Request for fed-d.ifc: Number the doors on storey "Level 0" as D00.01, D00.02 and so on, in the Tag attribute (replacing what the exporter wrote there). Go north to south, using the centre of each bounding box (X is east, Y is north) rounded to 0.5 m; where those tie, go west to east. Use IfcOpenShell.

First a look at what the model holds.

```python
import ifcopenshell
import ifcopenshell.util.element
import ifcopenshell.util.placement

model = ifcopenshell.open("fed-d.ifc")
print(model.schema)
storey = next(s for s in model.by_type("IfcBuildingStorey") if s.Name == "Level 0")
doors = [e for e in ifcopenshell.util.element.get_decomposition(storey) if e.is_a("IfcDoor")]
for e in sorted(doors, key=lambda e: e.id()):
    origin = ifcopenshell.util.placement.get_local_placement(e.ObjectPlacement)[:3, 3]
    print(e.id(), e.Tag, e.Name, origin.round(2) + 0.0, sep=" | ")
```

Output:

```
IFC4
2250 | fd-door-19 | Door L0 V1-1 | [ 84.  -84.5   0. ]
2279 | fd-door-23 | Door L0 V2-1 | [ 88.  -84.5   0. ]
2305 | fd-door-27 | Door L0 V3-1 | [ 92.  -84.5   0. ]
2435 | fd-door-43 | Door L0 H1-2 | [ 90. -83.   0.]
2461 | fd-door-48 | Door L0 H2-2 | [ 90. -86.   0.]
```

```python
import ifcopenshell
import ifcopenshell.geom
import ifcopenshell.util.element
import ifcopenshell.util.shape

model = ifcopenshell.open("fed-d.ifc")
settings = ifcopenshell.geom.settings()
settings.set("use-world-coords", True)


def centre(element):
    shape = ifcopenshell.geom.create_shape(settings, element)
    return ifcopenshell.util.shape.get_bbox_centroid(shape.geometry)


storey = next(s for s in model.by_type("IfcBuildingStorey") if s.Name == "Level 0")
doors = [e for e in ifcopenshell.util.element.get_decomposition(storey) if e.is_a("IfcDoor")]

# Insertion points can sit at a corner or the storey origin, so sort by the geometry (in metres).
centres = {e: centre(e) for e in doors}
doors.sort(key=lambda e: (-round(centres[e][1] / 0.5), centres[e][0]))

for i, e in enumerate(doors, start=1):
    number = f"D00.{i:02d}"
    e.Tag = number
    print(e.id(), number)

model.write("fed-d_updated.ifc")
```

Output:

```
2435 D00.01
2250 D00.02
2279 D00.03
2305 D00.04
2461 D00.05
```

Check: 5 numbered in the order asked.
